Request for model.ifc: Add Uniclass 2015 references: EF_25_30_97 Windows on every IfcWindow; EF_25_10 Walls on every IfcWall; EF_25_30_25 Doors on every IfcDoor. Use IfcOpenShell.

First a look at what the model holds.

```python
import ifcopenshell

model = ifcopenshell.open("model.ifc")
print(model.schema)
print("classifications:", [c.Name for c in model.by_type("IfcClassification")])
for ifc_class in ("IfcDoor", "IfcRoof", "IfcStair", "IfcWall", "IfcWindow"):
    print(ifc_class, len(model.by_type(ifc_class)))
```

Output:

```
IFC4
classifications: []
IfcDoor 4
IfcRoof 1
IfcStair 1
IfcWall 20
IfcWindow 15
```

```python
import ifcopenshell
import ifcopenshell.api.classification

model = ifcopenshell.open("model.ifc")

system = ifcopenshell.api.classification.add_classification(model, classification="Uniclass 2015")

codes = {
    "IfcWindow": ("EF_25_30_97", "Windows"),
    "IfcWall": ("EF_25_10", "Walls"),
    "IfcDoor": ("EF_25_30_25", "Doors"),
}
for ifc_class, (code, name) in codes.items():
    products = model.by_type(ifc_class)
    ifcopenshell.api.classification.add_reference(
        model, products=products, classification=system, identification=code, name=name
    )
    print(code, len(products))

model.write("model_edited.ifc")
```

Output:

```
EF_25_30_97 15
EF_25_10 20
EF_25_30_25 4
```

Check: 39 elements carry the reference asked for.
